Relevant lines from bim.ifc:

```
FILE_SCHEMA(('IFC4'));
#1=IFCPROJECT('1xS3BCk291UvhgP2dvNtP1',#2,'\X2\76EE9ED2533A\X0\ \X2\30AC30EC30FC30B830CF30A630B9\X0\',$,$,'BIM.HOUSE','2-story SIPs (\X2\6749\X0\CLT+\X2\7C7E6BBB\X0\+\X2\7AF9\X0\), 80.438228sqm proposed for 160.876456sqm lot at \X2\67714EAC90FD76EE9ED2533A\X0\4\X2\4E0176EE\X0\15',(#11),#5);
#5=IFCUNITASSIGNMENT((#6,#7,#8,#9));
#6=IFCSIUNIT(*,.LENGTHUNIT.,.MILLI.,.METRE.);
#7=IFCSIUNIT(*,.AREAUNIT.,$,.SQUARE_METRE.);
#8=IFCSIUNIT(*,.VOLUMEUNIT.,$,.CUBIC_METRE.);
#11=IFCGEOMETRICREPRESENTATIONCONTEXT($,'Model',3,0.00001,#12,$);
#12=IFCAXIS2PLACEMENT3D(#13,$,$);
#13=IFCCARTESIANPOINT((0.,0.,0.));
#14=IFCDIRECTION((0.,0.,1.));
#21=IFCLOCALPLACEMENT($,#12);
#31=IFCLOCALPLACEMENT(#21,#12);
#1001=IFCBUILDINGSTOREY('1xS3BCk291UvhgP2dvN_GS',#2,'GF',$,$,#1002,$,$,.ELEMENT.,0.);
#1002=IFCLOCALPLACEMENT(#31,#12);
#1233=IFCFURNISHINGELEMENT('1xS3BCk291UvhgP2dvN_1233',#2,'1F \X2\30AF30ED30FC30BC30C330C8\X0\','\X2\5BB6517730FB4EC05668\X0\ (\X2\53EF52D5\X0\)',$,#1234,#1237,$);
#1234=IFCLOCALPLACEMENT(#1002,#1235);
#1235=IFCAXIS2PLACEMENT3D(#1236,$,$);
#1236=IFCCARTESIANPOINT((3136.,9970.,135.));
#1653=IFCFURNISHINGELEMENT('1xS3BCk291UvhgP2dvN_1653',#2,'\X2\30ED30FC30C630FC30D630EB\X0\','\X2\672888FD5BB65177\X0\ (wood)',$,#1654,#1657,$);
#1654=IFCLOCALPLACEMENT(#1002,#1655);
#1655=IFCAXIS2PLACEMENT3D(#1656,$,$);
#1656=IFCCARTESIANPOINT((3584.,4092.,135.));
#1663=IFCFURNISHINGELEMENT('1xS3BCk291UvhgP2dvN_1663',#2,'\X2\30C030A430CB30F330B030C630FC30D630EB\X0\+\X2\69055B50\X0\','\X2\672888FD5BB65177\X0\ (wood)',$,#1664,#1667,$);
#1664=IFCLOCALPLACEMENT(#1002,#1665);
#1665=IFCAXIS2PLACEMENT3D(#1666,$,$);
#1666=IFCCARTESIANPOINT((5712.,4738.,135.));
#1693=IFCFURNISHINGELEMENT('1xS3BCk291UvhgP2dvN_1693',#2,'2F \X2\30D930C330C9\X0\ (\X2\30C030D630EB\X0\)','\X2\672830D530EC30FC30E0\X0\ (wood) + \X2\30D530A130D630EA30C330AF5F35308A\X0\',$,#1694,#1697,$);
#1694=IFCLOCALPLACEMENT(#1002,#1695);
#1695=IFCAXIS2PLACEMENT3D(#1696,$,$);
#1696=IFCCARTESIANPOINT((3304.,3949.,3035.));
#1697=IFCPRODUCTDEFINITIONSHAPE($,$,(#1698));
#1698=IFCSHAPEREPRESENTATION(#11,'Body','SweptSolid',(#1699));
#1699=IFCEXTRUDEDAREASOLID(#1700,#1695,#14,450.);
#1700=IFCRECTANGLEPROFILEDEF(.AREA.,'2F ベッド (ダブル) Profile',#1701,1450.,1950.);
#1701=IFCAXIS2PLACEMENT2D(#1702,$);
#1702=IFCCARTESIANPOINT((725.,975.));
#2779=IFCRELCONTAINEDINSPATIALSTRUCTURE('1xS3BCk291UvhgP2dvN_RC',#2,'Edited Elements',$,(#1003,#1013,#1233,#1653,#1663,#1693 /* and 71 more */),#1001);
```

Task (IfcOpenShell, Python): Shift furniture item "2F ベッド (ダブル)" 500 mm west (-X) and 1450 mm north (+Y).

```python
import ifcopenshell
import ifcopenshell.api.geometry
import ifcopenshell.util.placement
import ifcopenshell.util.unit

model = ifcopenshell.open("bim.ifc")
unit_scale = ifcopenshell.util.unit.calculate_unit_scale(model)

item = model.by_guid("1xS3BCk291UvhgP2dvN_1693")
matrix = ifcopenshell.util.placement.get_local_placement(item.ObjectPlacement)
matrix[0, 3] -= 0.5 / unit_scale
matrix[1, 3] += 1.45 / unit_scale
ifcopenshell.api.geometry.edit_object_placement(model, product=item, matrix=matrix, is_si=False)

print(ifcopenshell.util.placement.get_local_placement(item.ObjectPlacement).round(3) + 0.0)

model.write("bim_v2.ifc")
```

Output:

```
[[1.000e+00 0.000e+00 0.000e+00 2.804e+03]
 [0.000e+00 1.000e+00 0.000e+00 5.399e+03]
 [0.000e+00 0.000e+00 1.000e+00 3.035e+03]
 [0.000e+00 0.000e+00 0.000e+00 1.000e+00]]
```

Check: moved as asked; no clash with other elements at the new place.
